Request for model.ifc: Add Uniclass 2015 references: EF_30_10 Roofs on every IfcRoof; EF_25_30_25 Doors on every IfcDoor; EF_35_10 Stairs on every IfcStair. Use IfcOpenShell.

First a look at what the model holds.

```python
import ifcopenshell

model = ifcopenshell.open("model.ifc")
print(model.schema)
print("classifications:", [c.Name for c in model.by_type("IfcClassification")])
for ifc_class in ("IfcDoor", "IfcRoof", "IfcStair", "IfcWall", "IfcWindow"):
    print(ifc_class, len(model.by_type(ifc_class)))
```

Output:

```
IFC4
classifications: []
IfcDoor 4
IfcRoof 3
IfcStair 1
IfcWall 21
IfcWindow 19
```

```python
import ifcopenshell
import ifcopenshell.api.classification

model = ifcopenshell.open("model.ifc")

system = ifcopenshell.api.classification.add_classification(model, classification="Uniclass 2015")

codes = {
    "IfcRoof": ("EF_30_10", "Roofs"),
    "IfcDoor": ("EF_25_30_25", "Doors"),
    "IfcStair": ("EF_35_10", "Stairs"),
}
for ifc_class, (code, name) in codes.items():
    products = model.by_type(ifc_class)
    ifcopenshell.api.classification.add_reference(
        model, products=products, classification=system, identification=code, name=name
    )
    print(code, len(products))

model.write("model_updated.ifc")
```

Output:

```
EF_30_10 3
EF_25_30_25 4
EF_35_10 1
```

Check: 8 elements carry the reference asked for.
